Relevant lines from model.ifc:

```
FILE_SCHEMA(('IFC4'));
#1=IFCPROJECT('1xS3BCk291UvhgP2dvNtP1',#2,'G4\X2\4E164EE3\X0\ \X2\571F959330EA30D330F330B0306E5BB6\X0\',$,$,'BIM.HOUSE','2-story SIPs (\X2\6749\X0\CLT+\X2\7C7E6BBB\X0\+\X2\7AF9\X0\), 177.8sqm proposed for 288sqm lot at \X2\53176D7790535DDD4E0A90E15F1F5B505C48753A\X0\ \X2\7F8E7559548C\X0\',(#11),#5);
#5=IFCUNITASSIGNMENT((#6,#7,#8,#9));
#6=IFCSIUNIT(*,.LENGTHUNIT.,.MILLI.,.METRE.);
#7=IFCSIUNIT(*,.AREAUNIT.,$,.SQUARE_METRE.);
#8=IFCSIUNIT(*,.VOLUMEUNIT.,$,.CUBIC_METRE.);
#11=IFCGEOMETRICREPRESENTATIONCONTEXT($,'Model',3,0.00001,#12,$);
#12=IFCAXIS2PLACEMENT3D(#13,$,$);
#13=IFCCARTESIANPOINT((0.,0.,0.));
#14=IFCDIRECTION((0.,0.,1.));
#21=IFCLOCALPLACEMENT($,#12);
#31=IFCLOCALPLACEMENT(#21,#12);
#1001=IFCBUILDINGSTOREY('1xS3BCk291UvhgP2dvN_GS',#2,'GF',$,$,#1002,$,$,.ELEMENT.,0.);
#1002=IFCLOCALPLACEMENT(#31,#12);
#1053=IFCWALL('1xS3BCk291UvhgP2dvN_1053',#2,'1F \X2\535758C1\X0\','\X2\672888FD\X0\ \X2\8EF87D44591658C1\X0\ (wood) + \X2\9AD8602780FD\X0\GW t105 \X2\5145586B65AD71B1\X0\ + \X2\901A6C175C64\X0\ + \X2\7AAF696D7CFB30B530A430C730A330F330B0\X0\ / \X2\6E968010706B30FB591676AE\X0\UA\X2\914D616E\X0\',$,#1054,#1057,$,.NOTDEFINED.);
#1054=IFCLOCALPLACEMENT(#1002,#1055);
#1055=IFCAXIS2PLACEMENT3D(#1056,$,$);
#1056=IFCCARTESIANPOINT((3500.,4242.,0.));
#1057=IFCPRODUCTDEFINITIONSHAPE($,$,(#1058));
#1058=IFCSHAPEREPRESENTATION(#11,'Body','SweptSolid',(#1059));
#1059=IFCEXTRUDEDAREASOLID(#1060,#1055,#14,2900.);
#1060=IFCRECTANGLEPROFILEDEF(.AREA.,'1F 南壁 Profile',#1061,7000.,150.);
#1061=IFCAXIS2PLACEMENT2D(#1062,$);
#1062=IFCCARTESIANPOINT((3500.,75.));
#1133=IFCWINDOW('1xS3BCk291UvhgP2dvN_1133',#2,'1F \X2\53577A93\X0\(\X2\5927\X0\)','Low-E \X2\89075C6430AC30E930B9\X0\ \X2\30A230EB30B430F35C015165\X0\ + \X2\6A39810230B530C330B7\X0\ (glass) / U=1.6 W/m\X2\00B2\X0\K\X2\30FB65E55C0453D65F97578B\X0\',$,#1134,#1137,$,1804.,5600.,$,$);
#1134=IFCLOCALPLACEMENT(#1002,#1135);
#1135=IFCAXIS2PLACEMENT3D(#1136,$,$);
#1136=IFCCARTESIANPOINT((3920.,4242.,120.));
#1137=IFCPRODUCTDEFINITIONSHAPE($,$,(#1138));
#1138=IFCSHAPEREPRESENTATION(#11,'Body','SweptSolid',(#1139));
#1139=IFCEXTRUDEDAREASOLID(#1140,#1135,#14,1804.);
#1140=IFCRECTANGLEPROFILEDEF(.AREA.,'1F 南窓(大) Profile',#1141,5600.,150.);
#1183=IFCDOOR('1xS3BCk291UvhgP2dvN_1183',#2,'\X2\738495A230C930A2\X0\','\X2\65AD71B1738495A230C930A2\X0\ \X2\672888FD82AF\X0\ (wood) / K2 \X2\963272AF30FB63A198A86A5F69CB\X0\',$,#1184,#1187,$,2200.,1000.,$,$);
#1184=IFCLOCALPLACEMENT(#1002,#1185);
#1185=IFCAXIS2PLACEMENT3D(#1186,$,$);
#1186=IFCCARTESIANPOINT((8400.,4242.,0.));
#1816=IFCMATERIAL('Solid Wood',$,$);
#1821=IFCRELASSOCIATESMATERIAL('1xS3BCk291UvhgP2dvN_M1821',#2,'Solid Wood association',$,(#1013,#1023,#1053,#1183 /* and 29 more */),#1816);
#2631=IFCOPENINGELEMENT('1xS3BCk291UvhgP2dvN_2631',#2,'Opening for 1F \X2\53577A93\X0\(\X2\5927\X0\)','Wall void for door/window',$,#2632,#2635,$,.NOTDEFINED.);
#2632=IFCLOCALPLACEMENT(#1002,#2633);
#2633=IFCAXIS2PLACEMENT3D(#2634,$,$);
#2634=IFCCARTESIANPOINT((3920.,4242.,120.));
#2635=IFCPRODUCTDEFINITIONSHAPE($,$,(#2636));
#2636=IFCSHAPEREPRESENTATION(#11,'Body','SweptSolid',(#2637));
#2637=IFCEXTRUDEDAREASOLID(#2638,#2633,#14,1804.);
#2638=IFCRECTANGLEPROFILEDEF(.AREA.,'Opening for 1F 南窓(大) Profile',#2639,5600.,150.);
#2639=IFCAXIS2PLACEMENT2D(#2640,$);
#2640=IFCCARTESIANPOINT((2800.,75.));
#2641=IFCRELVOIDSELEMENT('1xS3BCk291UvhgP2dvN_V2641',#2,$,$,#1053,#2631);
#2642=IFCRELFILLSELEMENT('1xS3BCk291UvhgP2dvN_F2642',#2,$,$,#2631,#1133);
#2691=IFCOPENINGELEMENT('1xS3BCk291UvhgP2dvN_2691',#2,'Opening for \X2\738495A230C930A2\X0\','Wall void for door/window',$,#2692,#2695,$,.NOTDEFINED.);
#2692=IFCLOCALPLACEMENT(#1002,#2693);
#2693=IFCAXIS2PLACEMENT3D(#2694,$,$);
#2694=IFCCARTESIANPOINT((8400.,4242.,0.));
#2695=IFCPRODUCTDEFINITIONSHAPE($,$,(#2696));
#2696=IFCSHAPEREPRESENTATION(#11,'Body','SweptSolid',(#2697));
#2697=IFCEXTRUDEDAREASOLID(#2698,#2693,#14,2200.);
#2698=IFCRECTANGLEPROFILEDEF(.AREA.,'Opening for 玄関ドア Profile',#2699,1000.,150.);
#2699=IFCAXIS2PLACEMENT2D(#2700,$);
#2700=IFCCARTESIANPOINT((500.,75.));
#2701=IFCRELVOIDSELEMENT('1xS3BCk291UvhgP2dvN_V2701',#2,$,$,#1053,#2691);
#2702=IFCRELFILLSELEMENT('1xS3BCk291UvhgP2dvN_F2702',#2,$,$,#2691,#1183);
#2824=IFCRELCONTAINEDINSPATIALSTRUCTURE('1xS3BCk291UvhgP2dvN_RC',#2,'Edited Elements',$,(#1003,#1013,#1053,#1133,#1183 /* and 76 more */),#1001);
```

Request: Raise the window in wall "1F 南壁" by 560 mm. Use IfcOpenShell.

```python
import numpy as np
import ifcopenshell
import ifcopenshell.api.geometry
import ifcopenshell.util.placement
import ifcopenshell.util.unit

model = ifcopenshell.open("model.ifc")
unit_scale = ifcopenshell.util.unit.calculate_unit_scale(model)

window = model.by_guid("1xS3BCk291UvhgP2dvN_1133")
opening = window.FillsVoids[0].RelatingOpeningElement
dz = 0.56 / unit_scale

shift = np.array([0.0, 0.0, dz])
# The window is not placed relative to its opening, so move both.
for product in (opening, window):
    matrix = ifcopenshell.util.placement.get_local_placement(product.ObjectPlacement)
    matrix[:3, 3] += shift
    ifcopenshell.api.geometry.edit_object_placement(model, product=product, matrix=matrix, is_si=False)

print(f"moved by {dz * unit_scale:+.3f} m")

model.write("model_rev.ifc")
```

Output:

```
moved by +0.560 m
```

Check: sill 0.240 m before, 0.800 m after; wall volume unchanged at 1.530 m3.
